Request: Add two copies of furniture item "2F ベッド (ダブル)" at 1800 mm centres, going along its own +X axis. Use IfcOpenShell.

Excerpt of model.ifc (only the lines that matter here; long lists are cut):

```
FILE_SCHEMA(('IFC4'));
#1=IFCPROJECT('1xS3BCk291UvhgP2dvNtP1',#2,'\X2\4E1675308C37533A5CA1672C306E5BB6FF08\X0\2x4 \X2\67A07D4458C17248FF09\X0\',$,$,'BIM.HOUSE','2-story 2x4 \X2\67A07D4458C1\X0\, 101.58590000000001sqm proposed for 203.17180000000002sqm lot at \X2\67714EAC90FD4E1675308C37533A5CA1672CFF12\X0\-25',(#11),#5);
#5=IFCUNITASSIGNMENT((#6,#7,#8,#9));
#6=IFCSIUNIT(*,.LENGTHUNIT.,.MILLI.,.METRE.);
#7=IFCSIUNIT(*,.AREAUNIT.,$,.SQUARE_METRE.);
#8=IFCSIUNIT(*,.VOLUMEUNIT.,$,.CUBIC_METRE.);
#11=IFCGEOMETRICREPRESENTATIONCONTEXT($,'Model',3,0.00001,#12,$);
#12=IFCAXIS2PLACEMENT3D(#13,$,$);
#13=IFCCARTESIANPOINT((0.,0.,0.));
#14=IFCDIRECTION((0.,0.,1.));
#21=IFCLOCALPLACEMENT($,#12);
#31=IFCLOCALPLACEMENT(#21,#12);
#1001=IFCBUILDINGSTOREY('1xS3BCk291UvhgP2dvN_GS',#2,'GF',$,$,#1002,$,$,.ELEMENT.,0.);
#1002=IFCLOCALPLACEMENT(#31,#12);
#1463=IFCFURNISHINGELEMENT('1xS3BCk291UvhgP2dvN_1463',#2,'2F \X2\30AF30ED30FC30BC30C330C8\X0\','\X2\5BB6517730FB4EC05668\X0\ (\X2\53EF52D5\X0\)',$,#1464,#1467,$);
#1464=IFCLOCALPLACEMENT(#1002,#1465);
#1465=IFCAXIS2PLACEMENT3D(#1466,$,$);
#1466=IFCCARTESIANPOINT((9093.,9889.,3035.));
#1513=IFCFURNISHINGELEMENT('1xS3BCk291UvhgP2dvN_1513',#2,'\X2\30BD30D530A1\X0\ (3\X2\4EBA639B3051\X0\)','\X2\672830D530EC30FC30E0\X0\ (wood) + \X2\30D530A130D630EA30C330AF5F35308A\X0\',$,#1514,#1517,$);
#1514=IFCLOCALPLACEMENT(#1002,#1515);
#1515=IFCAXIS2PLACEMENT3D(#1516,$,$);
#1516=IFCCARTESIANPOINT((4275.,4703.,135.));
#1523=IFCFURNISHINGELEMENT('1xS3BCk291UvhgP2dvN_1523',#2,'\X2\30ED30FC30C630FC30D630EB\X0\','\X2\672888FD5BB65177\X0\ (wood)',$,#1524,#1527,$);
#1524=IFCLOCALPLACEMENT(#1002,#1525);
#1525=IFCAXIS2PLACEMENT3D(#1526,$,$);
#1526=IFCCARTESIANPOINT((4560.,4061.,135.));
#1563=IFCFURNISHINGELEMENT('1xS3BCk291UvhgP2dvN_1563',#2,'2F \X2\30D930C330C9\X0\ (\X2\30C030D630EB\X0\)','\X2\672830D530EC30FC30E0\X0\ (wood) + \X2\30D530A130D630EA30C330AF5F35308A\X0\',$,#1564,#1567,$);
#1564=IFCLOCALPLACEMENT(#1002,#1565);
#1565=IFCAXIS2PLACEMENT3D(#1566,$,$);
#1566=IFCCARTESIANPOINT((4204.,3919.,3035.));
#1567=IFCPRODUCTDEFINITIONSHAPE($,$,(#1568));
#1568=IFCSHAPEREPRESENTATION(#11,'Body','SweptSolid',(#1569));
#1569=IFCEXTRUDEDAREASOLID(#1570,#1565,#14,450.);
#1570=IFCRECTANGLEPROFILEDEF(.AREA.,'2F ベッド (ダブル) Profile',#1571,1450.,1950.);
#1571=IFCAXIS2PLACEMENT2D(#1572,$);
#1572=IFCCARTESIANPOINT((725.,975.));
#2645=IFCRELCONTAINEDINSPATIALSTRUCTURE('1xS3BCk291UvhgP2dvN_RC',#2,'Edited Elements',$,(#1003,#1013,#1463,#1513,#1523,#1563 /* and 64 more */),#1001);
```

```python
import ifcopenshell
import ifcopenshell.api.geometry
import ifcopenshell.api.root
import ifcopenshell.util.element
import ifcopenshell.util.placement
import ifcopenshell.util.unit

model = ifcopenshell.open("model.ifc")
unit_scale = ifcopenshell.util.unit.calculate_unit_scale(model)


def reuse_history(source, copy):
    """copy_class also copies each property set's owner history, people and application; keep the originals."""
    for rel in copy.IsDefinedBy:
        if rel.is_a("IfcRelDefinesByProperties") and (history := rel.RelatingPropertyDefinition.OwnerHistory):
            rel.RelatingPropertyDefinition.OwnerHistory = source.OwnerHistory
            ifcopenshell.util.element.remove_deep2(model, history)


source = model.by_guid("1xS3BCk291UvhgP2dvN_1563")
base = ifcopenshell.util.placement.get_local_placement(source.ObjectPlacement)
step = base[:3, 0] * 1.8 / unit_scale

for i in range(1, 3):
    copy = ifcopenshell.api.root.copy_class(model, product=source)
    copy.Representation = ifcopenshell.util.element.copy_deep(
        model, source.Representation, exclude=["IfcGeometricRepresentationContext", "IfcRepresentationMap"]
    )
    reuse_history(source, copy)
    matrix = base.copy()
    matrix[:3, 3] += i * step
    print("added at", matrix[:3, 3].round(3) + 0.0)
    ifcopenshell.api.geometry.edit_object_placement(model, product=copy, matrix=matrix, is_si=False)

model.write("model_rev.ifc")
```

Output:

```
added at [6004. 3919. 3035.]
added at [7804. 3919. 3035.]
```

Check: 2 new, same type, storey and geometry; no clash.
